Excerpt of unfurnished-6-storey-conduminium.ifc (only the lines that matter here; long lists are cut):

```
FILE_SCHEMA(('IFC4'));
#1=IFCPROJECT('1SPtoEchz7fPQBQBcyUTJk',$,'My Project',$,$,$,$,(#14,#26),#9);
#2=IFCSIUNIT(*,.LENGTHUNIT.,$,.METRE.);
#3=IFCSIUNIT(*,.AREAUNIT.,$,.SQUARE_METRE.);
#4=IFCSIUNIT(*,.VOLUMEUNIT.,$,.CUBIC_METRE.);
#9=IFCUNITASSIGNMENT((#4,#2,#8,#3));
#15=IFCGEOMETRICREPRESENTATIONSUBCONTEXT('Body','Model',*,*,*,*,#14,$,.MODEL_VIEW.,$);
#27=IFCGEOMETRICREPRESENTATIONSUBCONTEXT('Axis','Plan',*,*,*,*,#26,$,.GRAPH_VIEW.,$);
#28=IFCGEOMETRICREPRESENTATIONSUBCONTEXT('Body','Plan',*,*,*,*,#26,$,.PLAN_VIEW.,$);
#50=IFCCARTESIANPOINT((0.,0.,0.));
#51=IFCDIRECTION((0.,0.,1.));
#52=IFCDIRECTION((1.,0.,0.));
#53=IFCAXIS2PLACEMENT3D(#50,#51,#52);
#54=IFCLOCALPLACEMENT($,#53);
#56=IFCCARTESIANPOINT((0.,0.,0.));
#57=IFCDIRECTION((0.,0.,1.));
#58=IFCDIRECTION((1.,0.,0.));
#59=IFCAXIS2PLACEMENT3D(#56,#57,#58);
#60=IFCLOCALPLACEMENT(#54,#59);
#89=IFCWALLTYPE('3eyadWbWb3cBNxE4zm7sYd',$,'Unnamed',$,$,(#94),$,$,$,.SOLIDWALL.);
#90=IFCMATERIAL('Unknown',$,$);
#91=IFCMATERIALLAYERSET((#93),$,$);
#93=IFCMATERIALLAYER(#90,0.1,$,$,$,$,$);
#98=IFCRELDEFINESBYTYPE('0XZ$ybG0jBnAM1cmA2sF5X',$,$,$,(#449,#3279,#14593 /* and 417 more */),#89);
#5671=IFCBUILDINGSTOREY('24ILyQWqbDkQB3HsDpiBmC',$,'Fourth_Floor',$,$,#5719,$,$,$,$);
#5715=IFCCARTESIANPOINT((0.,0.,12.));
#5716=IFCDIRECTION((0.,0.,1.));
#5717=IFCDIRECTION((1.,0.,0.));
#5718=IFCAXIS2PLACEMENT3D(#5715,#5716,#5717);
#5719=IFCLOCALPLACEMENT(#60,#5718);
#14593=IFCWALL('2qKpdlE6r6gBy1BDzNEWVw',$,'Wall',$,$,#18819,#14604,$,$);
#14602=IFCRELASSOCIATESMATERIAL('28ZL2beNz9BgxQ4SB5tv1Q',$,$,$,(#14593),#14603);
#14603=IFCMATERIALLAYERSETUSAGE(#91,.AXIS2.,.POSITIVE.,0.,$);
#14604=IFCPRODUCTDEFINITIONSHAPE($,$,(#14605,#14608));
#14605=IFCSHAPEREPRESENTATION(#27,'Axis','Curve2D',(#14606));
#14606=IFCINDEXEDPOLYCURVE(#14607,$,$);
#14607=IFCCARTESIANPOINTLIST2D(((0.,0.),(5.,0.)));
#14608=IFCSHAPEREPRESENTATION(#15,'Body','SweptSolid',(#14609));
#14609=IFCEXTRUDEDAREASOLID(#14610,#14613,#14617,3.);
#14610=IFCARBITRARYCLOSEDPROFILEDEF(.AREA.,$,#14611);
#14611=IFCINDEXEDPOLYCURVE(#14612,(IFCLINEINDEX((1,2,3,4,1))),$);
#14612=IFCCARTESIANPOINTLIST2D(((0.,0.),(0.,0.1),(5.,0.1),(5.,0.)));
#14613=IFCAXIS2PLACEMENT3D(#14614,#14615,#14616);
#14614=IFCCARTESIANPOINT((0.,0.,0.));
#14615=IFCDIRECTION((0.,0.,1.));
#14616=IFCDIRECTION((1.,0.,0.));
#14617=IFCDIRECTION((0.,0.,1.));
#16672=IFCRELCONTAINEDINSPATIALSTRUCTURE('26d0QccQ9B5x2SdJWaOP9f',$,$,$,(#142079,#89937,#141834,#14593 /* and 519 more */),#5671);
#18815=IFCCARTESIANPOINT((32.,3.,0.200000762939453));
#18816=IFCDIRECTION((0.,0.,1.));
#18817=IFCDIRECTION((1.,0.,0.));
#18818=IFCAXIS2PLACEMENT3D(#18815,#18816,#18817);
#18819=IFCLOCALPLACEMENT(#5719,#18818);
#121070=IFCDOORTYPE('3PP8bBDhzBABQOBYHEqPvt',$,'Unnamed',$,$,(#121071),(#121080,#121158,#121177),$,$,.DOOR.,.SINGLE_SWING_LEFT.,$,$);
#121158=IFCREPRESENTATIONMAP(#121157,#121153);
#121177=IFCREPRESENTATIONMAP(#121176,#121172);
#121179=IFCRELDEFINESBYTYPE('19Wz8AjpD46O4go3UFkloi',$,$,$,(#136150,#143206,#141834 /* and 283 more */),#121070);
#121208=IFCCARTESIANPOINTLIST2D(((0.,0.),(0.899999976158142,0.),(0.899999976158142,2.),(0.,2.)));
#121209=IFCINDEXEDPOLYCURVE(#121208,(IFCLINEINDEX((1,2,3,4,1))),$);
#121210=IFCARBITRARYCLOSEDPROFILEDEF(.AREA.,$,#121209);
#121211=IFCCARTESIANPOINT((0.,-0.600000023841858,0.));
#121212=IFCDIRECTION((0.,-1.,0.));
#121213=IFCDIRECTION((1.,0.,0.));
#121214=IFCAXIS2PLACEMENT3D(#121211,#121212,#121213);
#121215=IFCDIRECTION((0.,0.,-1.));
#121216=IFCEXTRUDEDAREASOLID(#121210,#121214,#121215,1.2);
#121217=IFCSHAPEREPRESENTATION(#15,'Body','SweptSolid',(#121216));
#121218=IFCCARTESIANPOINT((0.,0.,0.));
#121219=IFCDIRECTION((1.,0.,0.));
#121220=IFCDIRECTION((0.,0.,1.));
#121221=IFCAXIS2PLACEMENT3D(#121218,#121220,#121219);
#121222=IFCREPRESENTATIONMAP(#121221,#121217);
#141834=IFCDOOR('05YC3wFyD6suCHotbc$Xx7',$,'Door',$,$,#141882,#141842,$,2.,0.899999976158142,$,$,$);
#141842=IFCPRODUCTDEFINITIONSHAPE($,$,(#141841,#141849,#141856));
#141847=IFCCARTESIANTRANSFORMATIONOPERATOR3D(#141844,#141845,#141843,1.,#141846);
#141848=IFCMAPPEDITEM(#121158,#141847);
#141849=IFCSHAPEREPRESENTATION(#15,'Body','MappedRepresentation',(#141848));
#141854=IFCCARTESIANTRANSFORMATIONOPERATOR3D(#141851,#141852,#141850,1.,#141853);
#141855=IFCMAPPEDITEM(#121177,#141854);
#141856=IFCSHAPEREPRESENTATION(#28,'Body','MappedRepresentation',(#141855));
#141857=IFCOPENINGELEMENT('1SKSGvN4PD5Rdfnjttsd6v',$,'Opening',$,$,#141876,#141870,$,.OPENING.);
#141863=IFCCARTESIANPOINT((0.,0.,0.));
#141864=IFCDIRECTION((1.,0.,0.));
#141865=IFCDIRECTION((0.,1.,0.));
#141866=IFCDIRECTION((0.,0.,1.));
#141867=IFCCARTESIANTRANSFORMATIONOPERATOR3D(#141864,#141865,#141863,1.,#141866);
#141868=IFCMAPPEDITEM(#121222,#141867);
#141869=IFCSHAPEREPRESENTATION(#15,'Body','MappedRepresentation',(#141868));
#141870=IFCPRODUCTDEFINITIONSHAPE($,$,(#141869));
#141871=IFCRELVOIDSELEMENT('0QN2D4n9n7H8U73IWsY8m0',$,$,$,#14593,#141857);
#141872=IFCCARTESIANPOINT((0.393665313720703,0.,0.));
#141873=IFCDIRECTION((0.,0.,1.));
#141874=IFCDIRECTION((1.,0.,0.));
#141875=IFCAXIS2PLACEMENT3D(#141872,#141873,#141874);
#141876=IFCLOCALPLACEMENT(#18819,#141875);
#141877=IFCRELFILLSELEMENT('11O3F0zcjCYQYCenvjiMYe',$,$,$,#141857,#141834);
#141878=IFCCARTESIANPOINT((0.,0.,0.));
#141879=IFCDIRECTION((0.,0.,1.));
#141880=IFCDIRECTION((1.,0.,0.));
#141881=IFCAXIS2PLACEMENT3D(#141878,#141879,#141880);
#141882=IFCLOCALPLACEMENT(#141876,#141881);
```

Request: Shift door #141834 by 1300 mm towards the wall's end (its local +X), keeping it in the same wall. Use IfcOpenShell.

```python
import ifcopenshell
import ifcopenshell.api.geometry
import ifcopenshell.util.placement
import ifcopenshell.util.unit

model = ifcopenshell.open("unfurnished-6-storey-conduminium.ifc")
unit_scale = ifcopenshell.util.unit.calculate_unit_scale(model)

door = model.by_id(141834)
opening = door.FillsVoids[0].RelatingOpeningElement
wall = opening.VoidsElements[0].RelatingBuildingElement

wall_matrix = ifcopenshell.util.placement.get_local_placement(wall.ObjectPlacement)
shift = wall_matrix[:3, 0] * 1.3 / unit_scale
before = ifcopenshell.util.placement.get_local_placement(door.ObjectPlacement)[:3, 3].copy()

# The door is placed relative to its opening, so it follows when the opening moves.
matrix = ifcopenshell.util.placement.get_local_placement(opening.ObjectPlacement)
matrix[:3, 3] += shift
ifcopenshell.api.geometry.edit_object_placement(
    model, product=opening, matrix=matrix, is_si=False, should_transform_children=True
)

after = ifcopenshell.util.placement.get_local_placement(door.ObjectPlacement)[:3, 3]
print("door moved by", (after - before).round(3) + 0.0)

model.write("unfurnished-6-storey-conduminium_v2.ifc")
```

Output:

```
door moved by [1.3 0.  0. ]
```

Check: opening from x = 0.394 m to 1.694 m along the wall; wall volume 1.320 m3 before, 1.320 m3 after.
